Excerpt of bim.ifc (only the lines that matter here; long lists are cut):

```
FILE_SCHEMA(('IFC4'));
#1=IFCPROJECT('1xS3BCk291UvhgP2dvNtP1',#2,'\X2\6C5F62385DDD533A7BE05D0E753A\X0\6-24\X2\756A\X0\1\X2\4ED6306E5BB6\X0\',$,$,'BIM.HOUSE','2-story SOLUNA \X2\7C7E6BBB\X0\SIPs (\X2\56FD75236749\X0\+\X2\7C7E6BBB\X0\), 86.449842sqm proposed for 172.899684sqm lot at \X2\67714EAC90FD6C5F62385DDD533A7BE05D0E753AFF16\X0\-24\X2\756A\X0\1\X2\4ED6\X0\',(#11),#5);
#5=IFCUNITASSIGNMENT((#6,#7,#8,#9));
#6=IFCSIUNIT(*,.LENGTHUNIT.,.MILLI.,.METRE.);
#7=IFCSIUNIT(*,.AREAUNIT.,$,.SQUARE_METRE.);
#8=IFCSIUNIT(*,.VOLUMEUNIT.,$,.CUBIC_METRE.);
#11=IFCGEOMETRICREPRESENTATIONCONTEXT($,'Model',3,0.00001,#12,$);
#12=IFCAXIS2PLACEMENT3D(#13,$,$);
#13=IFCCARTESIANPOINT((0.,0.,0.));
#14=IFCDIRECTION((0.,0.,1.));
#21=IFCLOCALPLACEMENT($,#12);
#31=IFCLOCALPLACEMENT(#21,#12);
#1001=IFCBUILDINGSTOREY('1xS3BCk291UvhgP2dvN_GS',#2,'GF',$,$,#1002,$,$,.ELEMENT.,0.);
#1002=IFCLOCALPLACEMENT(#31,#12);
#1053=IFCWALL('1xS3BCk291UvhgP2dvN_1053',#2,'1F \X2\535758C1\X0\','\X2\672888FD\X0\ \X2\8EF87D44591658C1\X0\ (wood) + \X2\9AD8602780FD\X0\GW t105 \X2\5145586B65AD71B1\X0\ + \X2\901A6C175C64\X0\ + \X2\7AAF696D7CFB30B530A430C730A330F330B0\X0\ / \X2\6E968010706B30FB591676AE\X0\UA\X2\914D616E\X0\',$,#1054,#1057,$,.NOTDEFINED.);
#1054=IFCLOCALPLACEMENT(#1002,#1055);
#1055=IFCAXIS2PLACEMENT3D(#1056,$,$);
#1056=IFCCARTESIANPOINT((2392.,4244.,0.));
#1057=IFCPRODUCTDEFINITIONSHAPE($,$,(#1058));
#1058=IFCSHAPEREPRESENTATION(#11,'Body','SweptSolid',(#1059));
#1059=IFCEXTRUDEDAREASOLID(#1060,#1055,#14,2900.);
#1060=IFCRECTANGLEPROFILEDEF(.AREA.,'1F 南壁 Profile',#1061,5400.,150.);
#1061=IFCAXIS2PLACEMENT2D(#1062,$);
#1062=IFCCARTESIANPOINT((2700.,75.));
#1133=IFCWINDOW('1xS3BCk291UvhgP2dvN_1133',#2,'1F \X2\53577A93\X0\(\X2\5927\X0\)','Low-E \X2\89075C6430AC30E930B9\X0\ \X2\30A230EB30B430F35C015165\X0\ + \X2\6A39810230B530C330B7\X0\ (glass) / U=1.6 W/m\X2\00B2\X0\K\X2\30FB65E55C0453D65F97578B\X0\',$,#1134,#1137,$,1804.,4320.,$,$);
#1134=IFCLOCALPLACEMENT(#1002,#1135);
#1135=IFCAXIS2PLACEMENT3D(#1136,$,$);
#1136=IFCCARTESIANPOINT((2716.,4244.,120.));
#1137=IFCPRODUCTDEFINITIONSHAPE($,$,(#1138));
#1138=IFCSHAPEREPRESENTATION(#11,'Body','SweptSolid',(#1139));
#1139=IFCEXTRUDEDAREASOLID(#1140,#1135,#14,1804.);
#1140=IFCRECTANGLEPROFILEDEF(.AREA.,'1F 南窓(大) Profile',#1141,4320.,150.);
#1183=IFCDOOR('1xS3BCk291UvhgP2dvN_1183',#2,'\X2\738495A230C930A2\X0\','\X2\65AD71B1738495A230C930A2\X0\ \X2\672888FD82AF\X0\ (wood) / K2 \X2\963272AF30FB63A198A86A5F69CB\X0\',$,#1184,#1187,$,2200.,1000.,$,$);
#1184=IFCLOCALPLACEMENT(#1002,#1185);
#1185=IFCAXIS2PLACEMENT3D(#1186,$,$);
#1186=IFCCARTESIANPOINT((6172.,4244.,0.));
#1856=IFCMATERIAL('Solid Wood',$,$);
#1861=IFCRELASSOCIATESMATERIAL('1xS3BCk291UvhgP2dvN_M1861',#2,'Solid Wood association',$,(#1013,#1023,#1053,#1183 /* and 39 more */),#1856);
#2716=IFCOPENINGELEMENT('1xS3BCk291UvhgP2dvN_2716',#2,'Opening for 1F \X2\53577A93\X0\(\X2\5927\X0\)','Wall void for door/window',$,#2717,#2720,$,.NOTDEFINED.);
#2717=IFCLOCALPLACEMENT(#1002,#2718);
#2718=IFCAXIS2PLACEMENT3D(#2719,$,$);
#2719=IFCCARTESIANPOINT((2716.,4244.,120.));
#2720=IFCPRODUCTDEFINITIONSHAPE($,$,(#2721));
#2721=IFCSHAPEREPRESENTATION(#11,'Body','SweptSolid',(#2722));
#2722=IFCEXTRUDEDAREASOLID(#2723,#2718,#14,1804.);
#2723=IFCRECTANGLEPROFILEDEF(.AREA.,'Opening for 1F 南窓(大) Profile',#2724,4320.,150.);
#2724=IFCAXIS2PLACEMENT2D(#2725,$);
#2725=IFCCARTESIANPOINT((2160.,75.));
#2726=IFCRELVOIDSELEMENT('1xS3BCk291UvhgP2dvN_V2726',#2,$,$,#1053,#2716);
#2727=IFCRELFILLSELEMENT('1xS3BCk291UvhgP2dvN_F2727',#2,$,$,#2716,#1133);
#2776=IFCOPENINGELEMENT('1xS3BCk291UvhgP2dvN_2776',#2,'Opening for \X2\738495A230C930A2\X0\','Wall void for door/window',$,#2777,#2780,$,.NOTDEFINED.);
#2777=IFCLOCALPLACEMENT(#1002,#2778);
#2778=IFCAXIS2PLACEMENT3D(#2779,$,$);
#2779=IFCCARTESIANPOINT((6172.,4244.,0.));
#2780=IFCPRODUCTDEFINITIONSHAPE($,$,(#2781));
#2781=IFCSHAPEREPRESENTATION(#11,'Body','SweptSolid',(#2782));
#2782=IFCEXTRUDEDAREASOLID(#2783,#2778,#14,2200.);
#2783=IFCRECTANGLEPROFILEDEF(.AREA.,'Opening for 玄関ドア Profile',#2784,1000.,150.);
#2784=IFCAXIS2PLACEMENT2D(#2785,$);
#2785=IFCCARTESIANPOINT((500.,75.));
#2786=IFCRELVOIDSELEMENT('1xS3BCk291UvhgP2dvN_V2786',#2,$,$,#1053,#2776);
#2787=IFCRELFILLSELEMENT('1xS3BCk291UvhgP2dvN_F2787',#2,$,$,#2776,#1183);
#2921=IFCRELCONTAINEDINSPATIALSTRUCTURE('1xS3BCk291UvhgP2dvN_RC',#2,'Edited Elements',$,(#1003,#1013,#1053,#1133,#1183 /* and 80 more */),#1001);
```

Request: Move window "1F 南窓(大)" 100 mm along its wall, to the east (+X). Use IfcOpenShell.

```python
import ifcopenshell
import ifcopenshell.api.geometry
import ifcopenshell.util.placement

model = ifcopenshell.open("bim.ifc")

window = model.by_guid("1xS3BCk291UvhgP2dvN_1133")
opening = window.FillsVoids[0].RelatingOpeningElement
wall = opening.VoidsElements[0].RelatingBuildingElement

wall_matrix = ifcopenshell.util.placement.get_local_placement(wall.ObjectPlacement)
shift = wall_matrix[:3, 0] * 100.0
before = ifcopenshell.util.placement.get_local_placement(window.ObjectPlacement)[:3, 3].copy()

# The window is not placed relative to its opening, so move both.
for product in (opening, window):
    matrix = ifcopenshell.util.placement.get_local_placement(product.ObjectPlacement)
    matrix[:3, 3] += shift
    ifcopenshell.api.geometry.edit_object_placement(model, product=product, matrix=matrix, is_si=False)

after = ifcopenshell.util.placement.get_local_placement(window.ObjectPlacement)[:3, 3]
print("window moved by", (after - before).round(3) + 0.0)

model.write("bim_rev.ifc")
```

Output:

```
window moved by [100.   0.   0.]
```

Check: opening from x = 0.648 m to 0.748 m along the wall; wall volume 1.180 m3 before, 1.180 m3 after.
